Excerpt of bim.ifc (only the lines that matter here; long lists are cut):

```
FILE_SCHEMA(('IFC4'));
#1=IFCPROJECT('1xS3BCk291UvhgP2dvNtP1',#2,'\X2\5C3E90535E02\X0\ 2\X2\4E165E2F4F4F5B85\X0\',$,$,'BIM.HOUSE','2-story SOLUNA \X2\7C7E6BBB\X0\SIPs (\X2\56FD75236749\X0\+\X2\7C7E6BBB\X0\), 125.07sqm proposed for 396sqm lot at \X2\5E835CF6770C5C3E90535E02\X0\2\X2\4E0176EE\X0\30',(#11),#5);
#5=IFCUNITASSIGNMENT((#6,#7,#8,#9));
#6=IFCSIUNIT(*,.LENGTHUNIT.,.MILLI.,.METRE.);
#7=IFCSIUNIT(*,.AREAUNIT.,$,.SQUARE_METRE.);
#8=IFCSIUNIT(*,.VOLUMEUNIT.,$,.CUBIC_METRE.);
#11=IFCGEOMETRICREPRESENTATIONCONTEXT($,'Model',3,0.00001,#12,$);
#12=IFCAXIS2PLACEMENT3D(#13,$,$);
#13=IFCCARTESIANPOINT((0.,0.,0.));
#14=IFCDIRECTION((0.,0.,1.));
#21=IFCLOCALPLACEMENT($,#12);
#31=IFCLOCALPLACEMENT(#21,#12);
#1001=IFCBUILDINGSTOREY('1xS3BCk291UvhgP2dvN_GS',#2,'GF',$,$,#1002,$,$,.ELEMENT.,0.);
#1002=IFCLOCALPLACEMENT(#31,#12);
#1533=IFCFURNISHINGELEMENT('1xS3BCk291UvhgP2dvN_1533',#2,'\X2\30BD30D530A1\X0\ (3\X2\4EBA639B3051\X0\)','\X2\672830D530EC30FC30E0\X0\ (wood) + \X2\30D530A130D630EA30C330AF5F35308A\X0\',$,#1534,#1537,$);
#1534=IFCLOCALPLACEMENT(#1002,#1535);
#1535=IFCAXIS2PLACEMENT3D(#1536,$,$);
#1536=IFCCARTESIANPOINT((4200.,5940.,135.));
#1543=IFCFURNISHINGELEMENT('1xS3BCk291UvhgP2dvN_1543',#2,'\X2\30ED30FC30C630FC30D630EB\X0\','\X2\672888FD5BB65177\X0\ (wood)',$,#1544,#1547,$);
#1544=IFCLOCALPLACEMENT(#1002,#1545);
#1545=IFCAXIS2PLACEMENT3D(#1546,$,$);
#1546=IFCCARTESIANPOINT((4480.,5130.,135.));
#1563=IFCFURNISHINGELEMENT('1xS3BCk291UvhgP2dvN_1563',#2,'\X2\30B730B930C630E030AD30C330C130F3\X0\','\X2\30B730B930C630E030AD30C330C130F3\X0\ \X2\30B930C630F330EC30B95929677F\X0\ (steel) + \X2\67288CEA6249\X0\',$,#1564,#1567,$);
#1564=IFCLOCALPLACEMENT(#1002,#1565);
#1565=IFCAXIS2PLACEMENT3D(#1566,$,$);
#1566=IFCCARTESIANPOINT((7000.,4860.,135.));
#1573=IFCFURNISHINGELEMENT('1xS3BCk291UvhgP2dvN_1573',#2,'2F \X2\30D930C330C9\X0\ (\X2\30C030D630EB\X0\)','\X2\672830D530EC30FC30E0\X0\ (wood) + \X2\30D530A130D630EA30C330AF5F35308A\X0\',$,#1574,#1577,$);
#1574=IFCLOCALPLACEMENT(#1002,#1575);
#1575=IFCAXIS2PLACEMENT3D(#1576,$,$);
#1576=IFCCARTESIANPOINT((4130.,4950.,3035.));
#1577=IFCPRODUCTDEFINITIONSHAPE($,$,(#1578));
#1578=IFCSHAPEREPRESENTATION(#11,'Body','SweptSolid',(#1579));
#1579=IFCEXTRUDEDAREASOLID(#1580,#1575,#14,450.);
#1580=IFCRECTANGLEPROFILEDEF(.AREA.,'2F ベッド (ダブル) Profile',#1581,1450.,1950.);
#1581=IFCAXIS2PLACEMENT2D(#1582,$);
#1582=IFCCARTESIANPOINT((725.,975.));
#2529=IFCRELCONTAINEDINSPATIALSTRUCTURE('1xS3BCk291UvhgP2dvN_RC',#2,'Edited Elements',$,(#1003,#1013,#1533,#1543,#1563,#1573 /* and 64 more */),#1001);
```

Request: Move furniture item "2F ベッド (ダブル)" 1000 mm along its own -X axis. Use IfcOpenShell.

```python
import ifcopenshell
import ifcopenshell.api.geometry
import ifcopenshell.util.placement
import ifcopenshell.util.unit

model = ifcopenshell.open("bim.ifc")
unit_scale = ifcopenshell.util.unit.calculate_unit_scale(model)

item = model.by_id(1573)
matrix = ifcopenshell.util.placement.get_local_placement(item.ObjectPlacement)
matrix[:3, 3] -= matrix[:3, 0] * 1 / unit_scale
ifcopenshell.api.geometry.edit_object_placement(model, product=item, matrix=matrix, is_si=False)

print(ifcopenshell.util.placement.get_local_placement(item.ObjectPlacement).round(3) + 0.0)

model.write("bim-out.ifc")
```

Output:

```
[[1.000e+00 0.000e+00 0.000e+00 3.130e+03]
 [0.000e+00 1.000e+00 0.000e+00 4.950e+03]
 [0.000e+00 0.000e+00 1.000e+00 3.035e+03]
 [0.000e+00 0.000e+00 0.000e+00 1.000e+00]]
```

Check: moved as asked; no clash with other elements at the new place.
